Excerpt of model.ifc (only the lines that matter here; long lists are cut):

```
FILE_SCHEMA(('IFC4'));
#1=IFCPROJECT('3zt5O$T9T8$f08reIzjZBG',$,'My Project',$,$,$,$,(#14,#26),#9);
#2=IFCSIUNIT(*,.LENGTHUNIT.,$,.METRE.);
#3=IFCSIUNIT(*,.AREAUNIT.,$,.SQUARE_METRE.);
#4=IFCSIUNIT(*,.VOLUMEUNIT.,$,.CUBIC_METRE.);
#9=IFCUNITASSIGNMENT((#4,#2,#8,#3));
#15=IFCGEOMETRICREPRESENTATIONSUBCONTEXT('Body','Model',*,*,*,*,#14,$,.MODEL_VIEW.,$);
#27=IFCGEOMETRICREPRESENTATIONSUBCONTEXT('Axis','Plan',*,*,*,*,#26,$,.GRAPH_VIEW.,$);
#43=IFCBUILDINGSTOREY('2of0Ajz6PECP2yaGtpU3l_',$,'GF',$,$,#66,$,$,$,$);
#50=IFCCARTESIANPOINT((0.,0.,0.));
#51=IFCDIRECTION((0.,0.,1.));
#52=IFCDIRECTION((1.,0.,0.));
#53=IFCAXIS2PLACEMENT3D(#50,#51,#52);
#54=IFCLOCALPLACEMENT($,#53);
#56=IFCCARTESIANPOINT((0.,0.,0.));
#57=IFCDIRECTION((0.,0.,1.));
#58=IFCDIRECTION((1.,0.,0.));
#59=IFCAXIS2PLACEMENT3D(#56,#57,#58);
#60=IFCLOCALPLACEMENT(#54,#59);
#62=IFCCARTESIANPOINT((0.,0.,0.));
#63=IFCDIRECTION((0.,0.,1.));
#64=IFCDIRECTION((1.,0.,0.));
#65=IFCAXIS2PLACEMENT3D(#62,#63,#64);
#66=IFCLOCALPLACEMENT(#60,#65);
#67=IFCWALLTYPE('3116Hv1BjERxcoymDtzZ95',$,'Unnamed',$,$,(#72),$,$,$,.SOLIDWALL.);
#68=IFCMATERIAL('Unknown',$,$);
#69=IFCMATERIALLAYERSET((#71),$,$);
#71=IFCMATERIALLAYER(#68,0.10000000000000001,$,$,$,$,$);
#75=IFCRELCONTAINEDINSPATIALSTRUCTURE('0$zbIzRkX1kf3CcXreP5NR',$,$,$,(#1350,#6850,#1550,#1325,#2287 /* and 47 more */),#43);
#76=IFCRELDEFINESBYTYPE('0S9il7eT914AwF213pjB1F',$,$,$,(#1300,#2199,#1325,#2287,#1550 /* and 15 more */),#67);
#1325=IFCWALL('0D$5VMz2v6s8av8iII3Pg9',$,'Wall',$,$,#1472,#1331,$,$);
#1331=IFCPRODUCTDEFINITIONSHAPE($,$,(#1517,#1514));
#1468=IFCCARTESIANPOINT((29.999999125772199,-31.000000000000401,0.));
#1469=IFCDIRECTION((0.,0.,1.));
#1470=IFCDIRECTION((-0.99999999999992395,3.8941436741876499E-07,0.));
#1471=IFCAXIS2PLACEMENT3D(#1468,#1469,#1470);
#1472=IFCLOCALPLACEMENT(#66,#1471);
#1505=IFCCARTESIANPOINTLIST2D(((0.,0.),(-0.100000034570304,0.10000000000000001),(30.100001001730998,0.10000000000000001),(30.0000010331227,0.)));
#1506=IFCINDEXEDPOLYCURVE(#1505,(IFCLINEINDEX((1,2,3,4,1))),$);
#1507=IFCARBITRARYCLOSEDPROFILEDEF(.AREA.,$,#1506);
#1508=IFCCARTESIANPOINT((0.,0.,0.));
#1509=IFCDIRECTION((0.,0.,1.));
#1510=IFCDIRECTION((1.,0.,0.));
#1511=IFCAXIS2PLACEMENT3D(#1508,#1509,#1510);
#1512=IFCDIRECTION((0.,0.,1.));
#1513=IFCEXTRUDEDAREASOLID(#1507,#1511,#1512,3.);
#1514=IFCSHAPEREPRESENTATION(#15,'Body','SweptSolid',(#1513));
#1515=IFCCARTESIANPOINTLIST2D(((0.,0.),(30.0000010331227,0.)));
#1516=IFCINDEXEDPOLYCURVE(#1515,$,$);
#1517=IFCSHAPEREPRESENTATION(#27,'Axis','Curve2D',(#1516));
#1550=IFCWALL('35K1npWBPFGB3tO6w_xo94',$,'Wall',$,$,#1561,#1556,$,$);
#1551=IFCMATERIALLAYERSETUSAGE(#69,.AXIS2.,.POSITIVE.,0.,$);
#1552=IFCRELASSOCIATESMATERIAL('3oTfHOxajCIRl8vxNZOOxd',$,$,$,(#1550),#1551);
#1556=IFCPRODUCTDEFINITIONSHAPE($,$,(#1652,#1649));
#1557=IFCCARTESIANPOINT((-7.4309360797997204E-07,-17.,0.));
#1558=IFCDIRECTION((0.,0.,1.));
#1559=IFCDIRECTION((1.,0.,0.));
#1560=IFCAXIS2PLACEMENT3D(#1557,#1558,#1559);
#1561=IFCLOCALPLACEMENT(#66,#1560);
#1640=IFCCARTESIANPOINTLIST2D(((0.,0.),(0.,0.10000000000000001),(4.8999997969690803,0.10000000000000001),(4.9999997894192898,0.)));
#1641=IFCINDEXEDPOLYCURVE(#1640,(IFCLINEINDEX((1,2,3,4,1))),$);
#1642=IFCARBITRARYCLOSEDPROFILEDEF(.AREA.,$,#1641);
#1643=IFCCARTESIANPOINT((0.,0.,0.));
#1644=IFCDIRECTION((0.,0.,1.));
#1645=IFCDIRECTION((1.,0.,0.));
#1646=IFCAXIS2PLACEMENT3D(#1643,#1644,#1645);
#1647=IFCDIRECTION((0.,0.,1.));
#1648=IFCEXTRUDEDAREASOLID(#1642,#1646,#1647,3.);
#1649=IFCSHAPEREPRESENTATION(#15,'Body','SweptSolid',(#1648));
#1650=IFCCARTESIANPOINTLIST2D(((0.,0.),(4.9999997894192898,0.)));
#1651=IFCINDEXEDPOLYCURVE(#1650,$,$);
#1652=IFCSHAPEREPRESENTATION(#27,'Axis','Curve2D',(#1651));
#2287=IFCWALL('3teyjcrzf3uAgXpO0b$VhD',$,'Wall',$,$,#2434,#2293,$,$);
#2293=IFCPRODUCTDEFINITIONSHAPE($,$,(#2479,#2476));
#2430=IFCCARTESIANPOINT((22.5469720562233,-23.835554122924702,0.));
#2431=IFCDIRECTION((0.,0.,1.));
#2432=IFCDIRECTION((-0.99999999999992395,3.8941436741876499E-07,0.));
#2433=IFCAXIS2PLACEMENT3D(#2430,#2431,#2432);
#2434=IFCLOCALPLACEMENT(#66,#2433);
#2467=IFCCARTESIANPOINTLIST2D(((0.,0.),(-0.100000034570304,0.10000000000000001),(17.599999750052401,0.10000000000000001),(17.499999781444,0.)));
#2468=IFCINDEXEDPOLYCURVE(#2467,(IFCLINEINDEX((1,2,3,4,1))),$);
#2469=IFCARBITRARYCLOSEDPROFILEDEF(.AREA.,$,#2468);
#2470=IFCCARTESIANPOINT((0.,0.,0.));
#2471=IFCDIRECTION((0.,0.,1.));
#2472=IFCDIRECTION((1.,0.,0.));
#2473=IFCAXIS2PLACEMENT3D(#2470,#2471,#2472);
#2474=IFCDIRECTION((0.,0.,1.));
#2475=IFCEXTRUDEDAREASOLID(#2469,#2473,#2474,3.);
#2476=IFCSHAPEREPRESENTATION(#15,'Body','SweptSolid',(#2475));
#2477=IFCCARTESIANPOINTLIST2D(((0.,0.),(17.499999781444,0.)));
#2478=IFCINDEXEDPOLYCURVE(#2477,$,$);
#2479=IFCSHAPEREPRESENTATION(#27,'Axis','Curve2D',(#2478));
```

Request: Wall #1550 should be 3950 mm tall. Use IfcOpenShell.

```python
import ifcopenshell
import ifcopenshell.geom
import ifcopenshell.util.representation
import ifcopenshell.util.shape
import ifcopenshell.util.unit

model = ifcopenshell.open("model.ifc")
unit_scale = ifcopenshell.util.unit.calculate_unit_scale(model)
settings = ifcopenshell.geom.settings()


def volume(element):
    """Net volume in cubic metres, openings subtracted."""
    shape = ifcopenshell.geom.create_shape(settings, element)
    return ifcopenshell.util.shape.get_volume(shape.geometry)


wall = model.by_guid("35K1npWBPFGB3tO6w_xo94")
before = volume(wall)

body = ifcopenshell.util.representation.get_representation(wall, "Model", "Body")
solid = body.Items[0]
old_height = solid.Depth
solid.Depth = 3.95 / unit_scale
after = volume(wall)

print(f"height {old_height:g} -> {solid.Depth:g}, volume {before:.3f} -> {after:.3f} m3")

model.write("model_edited.ifc")
```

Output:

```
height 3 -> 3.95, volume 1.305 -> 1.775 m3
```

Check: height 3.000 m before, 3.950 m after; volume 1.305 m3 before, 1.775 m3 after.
